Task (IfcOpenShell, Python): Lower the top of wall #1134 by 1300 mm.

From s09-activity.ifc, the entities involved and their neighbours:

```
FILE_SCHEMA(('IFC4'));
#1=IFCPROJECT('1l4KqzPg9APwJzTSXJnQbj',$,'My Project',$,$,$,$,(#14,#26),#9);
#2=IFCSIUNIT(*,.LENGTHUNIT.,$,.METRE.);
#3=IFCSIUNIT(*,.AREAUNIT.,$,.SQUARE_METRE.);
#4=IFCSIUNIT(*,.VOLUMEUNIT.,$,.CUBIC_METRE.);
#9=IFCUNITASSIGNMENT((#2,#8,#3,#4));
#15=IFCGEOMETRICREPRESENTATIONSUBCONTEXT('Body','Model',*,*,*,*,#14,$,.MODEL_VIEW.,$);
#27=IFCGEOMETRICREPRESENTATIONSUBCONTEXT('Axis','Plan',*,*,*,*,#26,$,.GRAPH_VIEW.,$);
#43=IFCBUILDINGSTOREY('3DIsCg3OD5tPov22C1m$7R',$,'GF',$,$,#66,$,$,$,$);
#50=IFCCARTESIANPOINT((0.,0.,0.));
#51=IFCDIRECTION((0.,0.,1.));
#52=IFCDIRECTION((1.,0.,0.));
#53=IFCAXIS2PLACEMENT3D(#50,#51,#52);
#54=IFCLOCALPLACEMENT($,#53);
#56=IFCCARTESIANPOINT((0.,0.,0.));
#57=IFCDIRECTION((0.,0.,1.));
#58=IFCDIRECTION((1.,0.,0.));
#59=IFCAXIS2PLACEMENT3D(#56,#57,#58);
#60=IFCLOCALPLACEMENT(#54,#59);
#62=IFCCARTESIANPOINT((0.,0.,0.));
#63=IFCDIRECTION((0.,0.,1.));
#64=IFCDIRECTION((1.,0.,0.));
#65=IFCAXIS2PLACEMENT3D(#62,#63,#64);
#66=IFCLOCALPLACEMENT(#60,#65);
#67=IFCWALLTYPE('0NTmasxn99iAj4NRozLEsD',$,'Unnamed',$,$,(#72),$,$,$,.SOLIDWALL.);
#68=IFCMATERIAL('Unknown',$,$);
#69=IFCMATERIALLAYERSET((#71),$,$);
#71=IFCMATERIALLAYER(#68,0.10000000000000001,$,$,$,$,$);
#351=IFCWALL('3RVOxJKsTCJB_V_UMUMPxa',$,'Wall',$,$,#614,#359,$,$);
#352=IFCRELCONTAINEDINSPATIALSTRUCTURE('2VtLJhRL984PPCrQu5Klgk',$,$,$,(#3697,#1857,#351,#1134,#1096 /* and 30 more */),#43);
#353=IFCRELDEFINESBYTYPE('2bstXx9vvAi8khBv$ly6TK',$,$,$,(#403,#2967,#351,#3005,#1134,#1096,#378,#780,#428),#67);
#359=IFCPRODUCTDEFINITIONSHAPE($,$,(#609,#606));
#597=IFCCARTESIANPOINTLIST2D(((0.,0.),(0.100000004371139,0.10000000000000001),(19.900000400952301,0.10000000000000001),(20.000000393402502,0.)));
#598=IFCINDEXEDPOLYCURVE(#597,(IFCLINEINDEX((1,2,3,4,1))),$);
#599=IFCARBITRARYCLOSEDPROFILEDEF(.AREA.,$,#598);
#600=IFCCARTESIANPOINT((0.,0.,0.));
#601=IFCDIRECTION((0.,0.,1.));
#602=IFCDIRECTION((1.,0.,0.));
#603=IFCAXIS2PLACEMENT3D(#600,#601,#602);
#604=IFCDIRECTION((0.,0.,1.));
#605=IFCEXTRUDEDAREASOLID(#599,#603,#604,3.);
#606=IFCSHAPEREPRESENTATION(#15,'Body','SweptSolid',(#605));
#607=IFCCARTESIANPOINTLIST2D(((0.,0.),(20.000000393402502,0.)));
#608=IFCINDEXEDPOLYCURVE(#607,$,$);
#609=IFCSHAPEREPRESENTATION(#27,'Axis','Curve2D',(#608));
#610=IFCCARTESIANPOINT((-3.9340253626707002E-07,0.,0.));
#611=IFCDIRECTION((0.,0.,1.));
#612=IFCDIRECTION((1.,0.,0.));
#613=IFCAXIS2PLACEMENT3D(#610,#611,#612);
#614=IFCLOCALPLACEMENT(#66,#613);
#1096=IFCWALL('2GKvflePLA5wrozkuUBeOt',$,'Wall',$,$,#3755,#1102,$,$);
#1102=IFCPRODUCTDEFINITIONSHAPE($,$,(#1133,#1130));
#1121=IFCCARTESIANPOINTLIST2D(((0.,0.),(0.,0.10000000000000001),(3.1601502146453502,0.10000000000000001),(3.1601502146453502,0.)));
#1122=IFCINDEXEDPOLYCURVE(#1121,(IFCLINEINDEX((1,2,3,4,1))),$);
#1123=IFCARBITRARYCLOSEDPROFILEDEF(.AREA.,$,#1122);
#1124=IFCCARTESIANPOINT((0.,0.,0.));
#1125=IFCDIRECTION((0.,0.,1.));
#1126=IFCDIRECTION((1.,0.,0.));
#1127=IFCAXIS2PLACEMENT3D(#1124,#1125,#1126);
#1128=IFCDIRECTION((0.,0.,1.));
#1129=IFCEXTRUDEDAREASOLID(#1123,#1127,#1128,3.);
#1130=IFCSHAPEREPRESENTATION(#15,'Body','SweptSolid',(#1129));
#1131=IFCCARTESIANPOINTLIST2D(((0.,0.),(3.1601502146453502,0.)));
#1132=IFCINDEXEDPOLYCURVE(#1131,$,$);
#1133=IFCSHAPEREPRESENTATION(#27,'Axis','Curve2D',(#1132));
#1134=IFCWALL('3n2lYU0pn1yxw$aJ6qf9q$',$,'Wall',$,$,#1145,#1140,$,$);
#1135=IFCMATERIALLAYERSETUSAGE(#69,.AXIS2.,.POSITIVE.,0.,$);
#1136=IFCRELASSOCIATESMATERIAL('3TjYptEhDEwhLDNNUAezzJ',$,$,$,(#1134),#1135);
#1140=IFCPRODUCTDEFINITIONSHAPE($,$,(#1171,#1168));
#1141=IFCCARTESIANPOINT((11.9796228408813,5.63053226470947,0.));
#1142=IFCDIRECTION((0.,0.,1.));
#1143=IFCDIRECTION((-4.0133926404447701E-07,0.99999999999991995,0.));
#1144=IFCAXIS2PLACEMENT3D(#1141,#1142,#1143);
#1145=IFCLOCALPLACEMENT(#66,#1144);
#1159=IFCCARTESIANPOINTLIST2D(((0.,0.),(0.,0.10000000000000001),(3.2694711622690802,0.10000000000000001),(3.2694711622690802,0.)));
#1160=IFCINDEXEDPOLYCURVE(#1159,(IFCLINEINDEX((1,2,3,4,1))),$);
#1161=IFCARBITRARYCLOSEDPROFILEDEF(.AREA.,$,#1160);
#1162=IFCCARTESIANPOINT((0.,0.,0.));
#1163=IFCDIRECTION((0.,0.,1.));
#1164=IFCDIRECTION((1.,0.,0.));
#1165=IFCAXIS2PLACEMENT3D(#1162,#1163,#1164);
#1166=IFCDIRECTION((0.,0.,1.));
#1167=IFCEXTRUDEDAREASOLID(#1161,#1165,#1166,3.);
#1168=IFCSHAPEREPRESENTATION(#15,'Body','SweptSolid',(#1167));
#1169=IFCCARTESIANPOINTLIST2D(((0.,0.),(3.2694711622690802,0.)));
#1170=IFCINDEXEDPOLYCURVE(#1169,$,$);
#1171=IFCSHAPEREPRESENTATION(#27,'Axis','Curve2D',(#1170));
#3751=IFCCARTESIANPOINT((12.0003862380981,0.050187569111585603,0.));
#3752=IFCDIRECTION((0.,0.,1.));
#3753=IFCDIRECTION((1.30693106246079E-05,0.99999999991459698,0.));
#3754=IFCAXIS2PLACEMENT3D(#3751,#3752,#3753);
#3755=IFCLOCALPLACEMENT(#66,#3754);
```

```python
import ifcopenshell
import ifcopenshell.geom
import ifcopenshell.util.representation
import ifcopenshell.util.shape
import ifcopenshell.util.unit

model = ifcopenshell.open("s09-activity.ifc")
unit_scale = ifcopenshell.util.unit.calculate_unit_scale(model)
settings = ifcopenshell.geom.settings()


def volume(element):
    """Net volume in cubic metres, openings subtracted."""
    shape = ifcopenshell.geom.create_shape(settings, element)
    return ifcopenshell.util.shape.get_volume(shape.geometry)


wall = model.by_guid("3n2lYU0pn1yxw$aJ6qf9q$")
before = volume(wall)

body = ifcopenshell.util.representation.get_representation(wall, "Model", "Body")
solid = body.Items[0]
old_height = solid.Depth
solid.Depth -= 1.3 / unit_scale
after = volume(wall)

print(f"height {old_height:g} -> {solid.Depth:g}, volume {before:.3f} -> {after:.3f} m3")

model.write("s09-activity_rev.ifc")
```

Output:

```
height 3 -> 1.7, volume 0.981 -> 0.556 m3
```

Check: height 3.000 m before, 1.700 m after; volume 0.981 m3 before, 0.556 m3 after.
